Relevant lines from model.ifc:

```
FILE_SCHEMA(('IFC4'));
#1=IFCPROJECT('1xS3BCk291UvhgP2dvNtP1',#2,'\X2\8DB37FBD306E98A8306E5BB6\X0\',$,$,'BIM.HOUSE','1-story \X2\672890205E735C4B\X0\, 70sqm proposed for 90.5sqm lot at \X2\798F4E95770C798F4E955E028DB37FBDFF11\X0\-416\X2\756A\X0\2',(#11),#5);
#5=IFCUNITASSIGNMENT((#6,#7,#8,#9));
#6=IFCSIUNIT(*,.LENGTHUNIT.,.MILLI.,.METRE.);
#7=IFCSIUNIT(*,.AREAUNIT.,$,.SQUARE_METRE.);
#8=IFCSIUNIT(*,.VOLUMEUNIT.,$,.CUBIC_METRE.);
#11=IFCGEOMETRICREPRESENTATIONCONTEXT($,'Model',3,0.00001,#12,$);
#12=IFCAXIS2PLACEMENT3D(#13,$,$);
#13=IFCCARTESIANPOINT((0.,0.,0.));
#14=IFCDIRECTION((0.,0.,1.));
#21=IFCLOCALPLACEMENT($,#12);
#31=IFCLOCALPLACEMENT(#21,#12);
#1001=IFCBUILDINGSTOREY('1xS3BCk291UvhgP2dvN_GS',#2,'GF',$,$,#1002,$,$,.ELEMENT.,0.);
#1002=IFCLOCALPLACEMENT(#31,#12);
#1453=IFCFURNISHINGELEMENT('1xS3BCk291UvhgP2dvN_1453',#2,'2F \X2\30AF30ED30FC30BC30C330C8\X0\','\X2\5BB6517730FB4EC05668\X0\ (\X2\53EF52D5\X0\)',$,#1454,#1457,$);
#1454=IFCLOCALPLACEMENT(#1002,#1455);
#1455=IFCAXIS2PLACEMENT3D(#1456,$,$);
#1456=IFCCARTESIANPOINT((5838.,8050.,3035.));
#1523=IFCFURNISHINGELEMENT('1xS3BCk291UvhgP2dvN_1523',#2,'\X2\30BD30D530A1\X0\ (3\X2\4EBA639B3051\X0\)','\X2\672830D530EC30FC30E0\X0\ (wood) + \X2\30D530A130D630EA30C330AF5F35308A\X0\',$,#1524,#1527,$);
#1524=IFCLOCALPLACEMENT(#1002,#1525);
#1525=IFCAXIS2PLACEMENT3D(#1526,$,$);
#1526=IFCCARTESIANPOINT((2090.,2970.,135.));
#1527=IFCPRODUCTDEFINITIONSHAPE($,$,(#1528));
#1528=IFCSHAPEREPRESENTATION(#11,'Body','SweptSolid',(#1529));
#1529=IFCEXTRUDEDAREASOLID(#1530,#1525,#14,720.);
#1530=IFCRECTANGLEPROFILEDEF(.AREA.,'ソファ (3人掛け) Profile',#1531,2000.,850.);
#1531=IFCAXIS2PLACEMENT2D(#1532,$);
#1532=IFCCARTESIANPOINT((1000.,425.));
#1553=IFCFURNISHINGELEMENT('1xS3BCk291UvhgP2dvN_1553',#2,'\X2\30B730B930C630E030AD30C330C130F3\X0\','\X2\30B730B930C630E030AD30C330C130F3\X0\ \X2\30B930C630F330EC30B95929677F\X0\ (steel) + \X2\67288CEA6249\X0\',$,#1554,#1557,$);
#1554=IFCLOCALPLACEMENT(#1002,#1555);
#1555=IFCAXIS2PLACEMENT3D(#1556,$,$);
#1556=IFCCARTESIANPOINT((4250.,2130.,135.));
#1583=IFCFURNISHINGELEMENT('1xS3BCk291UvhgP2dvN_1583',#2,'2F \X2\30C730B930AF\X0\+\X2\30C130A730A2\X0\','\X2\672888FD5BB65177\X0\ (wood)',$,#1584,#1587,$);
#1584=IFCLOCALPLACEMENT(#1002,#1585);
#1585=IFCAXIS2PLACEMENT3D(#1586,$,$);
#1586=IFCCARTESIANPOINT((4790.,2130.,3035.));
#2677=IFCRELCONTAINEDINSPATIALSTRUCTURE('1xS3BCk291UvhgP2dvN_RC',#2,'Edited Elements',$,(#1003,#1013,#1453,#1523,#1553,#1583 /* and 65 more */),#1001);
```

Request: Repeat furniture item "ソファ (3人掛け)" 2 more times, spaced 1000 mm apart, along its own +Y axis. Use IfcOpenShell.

```python
import ifcopenshell
import ifcopenshell.api.geometry
import ifcopenshell.api.root
import ifcopenshell.util.element
import ifcopenshell.util.placement

model = ifcopenshell.open("model.ifc")


def reuse_history(source, copy):
    """copy_class also copies each property set's owner history, people and application; keep the originals."""
    for rel in copy.IsDefinedBy:
        if rel.is_a("IfcRelDefinesByProperties") and (history := rel.RelatingPropertyDefinition.OwnerHistory):
            rel.RelatingPropertyDefinition.OwnerHistory = source.OwnerHistory
            ifcopenshell.util.element.remove_deep2(model, history)


source = model.by_id(1523)
base = ifcopenshell.util.placement.get_local_placement(source.ObjectPlacement)
step = base[:3, 1] * 1000.0

for i in range(1, 3):
    copy = ifcopenshell.api.root.copy_class(model, product=source)
    copy.Representation = ifcopenshell.util.element.copy_deep(
        model, source.Representation, exclude=["IfcGeometricRepresentationContext", "IfcRepresentationMap"]
    )
    reuse_history(source, copy)
    matrix = base.copy()
    matrix[:3, 3] += i * step
    print("added at", matrix[:3, 3].round(3) + 0.0)
    ifcopenshell.api.geometry.edit_object_placement(model, product=copy, matrix=matrix, is_si=False)

model.write("model-out.ifc")
```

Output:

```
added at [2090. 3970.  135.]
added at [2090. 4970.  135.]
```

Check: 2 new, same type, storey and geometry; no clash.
